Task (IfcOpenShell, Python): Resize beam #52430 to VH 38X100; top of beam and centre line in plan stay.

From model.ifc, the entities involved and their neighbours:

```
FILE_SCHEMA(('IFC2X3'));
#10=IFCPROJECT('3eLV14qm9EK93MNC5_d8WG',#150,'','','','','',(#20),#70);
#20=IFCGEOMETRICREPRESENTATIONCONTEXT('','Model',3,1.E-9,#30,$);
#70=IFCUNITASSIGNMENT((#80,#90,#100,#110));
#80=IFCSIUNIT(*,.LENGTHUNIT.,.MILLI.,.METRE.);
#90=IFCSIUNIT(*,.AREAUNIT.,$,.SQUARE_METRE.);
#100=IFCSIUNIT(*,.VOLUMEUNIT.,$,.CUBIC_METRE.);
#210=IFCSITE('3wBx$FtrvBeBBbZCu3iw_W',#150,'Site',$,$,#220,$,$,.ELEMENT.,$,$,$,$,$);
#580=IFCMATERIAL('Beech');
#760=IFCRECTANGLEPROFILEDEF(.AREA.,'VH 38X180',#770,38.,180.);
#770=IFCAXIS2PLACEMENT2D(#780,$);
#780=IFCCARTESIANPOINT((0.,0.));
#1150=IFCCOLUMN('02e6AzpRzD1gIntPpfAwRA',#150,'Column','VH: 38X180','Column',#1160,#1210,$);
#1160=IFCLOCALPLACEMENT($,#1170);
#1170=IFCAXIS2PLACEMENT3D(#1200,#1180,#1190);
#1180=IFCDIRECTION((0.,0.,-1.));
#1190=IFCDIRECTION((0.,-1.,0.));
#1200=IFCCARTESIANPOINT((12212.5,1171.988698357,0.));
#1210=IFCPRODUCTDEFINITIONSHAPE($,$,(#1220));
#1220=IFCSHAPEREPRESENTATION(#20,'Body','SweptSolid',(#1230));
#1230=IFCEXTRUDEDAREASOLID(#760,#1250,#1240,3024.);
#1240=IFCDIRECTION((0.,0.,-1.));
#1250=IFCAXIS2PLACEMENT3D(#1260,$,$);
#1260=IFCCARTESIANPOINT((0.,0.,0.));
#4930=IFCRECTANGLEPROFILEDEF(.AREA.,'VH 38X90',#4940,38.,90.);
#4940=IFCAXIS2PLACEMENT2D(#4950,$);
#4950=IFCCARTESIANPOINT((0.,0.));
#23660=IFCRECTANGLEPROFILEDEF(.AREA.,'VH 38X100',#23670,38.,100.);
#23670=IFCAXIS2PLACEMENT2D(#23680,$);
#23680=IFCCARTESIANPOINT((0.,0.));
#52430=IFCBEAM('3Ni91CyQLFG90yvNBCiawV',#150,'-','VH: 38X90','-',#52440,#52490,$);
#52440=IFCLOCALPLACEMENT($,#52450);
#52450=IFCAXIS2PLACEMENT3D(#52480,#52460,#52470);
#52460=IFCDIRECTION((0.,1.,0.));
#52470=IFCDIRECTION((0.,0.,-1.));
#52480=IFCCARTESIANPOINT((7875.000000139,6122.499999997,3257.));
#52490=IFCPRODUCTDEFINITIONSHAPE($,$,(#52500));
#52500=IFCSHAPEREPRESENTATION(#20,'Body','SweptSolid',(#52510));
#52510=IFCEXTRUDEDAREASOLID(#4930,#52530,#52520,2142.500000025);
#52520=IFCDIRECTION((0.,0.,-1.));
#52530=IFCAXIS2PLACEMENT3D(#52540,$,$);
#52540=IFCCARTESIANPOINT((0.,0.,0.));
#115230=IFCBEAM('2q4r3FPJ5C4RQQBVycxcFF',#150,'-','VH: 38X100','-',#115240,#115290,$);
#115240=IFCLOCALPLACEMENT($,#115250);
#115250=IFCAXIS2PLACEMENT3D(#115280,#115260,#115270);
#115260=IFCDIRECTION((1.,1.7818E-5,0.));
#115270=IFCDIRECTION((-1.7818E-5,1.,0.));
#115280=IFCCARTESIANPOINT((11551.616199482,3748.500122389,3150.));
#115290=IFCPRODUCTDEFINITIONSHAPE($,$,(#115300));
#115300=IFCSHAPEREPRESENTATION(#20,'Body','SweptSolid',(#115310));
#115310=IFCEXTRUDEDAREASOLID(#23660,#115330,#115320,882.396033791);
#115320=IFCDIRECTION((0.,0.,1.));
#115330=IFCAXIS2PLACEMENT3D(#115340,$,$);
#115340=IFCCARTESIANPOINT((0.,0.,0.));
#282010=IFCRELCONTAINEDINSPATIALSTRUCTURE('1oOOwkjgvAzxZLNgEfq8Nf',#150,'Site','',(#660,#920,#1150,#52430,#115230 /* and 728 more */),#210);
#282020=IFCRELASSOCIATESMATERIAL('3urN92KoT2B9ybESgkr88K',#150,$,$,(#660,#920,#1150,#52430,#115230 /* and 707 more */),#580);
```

```python
import ifcopenshell
import ifcopenshell.util.element

model = ifcopenshell.open("model.ifc")

member = model.by_guid("3Ni91CyQLFG90yvNBCiawV")
source = next(p for p in model.by_type("IfcRectangleProfileDef") if p.ProfileName == "VH 38X100")

body = next(r for r in member.Representation.Representations if r.RepresentationIdentifier == "Body")
solid = body.Items[0]
old_profile = solid.SweptArea

# Copy the section's sizes but keep this member's own profile position.
profile = ifcopenshell.util.element.copy(model, source)
# Profiles are centred, so shift by half the change in depth to hold the top.
shift = (old_profile.XDim - profile.XDim) / 2
x, y = old_profile.Position.Location.Coordinates
up = (-1.0, 0.0)  # upwards, in the solid's own plane
location = model.createIfcCartesianPoint((x + up[0] * shift, y + up[1] * shift))
profile.Position = model.createIfcAxis2Placement2D(location, old_profile.Position.RefDirection)
solid.SweptArea = profile
if not model.get_total_inverses(old_profile):
    ifcopenshell.util.element.remove_deep2(model, old_profile)

print(solid.SweptArea)

model.write("model-out.ifc")
```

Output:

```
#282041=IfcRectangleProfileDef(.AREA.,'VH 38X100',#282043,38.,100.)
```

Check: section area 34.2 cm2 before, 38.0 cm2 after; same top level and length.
